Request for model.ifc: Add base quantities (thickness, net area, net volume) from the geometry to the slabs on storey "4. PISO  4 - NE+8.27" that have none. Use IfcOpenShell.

First a look at what the model holds.

```python
import ifcopenshell
import ifcopenshell.util.element
import ifcopenshell.util.unit

model = ifcopenshell.open("model.ifc")
print(model.schema)
for unit_type in ("LENGTHUNIT", "AREAUNIT", "VOLUMEUNIT"):
    print(unit_type, ifcopenshell.util.unit.calculate_unit_scale(model, unit_type))
storey = next(s for s in model.by_type("IfcBuildingStorey") if s.Name == "4. PISO  4 - NE+8.27")
slabs = [e for e in ifcopenshell.util.element.get_decomposition(storey) if e.is_a("IfcSlab")]
for e in sorted(slabs, key=lambda e: e.id()):
    print(e.id(), e.is_a(), e.Name, list(ifcopenshell.util.element.get_psets(e, qtos_only=True)), sep=" | ")
```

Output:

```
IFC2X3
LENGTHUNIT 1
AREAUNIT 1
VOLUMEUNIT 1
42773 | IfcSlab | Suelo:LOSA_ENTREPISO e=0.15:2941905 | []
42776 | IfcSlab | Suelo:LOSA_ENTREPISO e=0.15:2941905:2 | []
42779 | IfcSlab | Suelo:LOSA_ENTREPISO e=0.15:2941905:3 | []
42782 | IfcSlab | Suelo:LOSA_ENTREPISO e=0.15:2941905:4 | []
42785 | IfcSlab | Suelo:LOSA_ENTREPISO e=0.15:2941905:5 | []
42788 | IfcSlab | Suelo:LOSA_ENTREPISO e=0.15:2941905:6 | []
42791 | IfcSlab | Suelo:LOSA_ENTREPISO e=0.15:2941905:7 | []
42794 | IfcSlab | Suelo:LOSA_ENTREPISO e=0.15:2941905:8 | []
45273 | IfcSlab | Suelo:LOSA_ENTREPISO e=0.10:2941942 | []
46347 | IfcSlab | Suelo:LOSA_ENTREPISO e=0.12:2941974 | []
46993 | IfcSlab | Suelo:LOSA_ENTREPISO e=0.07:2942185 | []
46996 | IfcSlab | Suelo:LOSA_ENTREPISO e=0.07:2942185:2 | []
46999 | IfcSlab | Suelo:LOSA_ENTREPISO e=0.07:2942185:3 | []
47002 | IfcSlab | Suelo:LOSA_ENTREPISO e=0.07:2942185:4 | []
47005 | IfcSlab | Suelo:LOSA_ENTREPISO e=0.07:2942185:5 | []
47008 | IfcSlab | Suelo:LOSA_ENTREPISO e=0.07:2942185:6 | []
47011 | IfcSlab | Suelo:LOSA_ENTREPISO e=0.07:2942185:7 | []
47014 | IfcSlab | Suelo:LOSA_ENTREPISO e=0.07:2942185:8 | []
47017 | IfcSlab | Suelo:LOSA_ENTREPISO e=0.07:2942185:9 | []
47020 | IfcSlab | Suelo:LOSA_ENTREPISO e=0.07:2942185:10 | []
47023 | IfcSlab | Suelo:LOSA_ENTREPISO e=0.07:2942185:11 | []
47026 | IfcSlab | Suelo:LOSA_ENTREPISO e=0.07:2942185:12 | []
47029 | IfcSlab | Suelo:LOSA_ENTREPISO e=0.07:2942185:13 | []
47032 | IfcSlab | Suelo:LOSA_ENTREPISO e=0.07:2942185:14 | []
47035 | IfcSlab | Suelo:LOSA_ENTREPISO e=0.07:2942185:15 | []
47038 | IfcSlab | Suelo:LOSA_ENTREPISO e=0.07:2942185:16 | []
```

```python
import ifcopenshell
import ifcopenshell.api.pset
import ifcopenshell.geom
import ifcopenshell.util.element
import ifcopenshell.util.shape
import ifcopenshell.util.unit

model = ifcopenshell.open("model.ifc")
unit_scale = ifcopenshell.util.unit.calculate_unit_scale(model)
area_scale = ifcopenshell.util.unit.calculate_unit_scale(model, "AREAUNIT")
volume_scale = ifcopenshell.util.unit.calculate_unit_scale(model, "VOLUMEUNIT")
settings = ifcopenshell.geom.settings()

storey = next(s for s in model.by_type("IfcBuildingStorey") if s.Name == "4. PISO  4 - NE+8.27")
slabs = [e for e in ifcopenshell.util.element.get_decomposition(storey) if e.is_a("IfcSlab")]

for e in sorted(slabs, key=lambda e: e.id()):
    if ifcopenshell.util.element.get_psets(e, qtos_only=True, should_inherit=False):
        continue
    # Geometry comes back in metres, in the element's own axes.
    shape = ifcopenshell.geom.create_shape(settings, e)
    values = {
        "Width": ifcopenshell.util.shape.get_z(shape.geometry) / unit_scale,
        "NetArea": ifcopenshell.util.shape.get_footprint_area(shape.geometry) / area_scale,
        "NetVolume": ifcopenshell.util.shape.get_volume(shape.geometry) / volume_scale,
    }
    qto = ifcopenshell.api.pset.add_qto(model, product=e, name="BaseQuantities")
    ifcopenshell.api.pset.edit_qto(model, qto=qto, properties=values)
    print(e.id(), {k: round(v, 3) for k, v in values.items()})

model.write("model_v2.ifc")
```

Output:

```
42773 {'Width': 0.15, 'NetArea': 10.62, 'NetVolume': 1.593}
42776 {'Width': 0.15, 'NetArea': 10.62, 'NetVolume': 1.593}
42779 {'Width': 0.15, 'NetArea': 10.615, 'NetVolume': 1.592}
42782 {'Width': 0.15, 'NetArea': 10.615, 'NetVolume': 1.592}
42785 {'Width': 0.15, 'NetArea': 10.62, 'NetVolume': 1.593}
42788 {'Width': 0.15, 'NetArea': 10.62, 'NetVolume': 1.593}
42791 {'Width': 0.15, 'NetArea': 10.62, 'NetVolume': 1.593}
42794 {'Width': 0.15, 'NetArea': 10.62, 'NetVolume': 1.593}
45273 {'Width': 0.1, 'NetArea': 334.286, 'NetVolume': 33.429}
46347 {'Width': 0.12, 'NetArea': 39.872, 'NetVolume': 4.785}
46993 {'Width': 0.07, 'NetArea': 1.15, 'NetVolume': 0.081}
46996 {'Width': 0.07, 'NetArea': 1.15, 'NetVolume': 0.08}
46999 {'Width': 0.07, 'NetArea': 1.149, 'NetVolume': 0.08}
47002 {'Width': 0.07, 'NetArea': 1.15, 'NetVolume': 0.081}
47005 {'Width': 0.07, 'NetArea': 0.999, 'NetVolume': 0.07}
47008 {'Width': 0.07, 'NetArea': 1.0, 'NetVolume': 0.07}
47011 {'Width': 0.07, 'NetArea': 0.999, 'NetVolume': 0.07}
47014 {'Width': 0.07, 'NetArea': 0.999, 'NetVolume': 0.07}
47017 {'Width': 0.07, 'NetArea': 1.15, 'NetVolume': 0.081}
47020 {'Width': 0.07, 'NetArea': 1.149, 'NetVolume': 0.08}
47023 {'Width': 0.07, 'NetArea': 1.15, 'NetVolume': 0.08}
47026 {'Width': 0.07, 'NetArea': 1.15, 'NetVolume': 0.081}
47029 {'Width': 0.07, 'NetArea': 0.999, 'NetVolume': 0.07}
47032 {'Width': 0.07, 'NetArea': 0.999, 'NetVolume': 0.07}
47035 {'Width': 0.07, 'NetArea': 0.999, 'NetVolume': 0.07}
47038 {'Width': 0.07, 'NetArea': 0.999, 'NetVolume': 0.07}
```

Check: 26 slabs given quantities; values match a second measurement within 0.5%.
